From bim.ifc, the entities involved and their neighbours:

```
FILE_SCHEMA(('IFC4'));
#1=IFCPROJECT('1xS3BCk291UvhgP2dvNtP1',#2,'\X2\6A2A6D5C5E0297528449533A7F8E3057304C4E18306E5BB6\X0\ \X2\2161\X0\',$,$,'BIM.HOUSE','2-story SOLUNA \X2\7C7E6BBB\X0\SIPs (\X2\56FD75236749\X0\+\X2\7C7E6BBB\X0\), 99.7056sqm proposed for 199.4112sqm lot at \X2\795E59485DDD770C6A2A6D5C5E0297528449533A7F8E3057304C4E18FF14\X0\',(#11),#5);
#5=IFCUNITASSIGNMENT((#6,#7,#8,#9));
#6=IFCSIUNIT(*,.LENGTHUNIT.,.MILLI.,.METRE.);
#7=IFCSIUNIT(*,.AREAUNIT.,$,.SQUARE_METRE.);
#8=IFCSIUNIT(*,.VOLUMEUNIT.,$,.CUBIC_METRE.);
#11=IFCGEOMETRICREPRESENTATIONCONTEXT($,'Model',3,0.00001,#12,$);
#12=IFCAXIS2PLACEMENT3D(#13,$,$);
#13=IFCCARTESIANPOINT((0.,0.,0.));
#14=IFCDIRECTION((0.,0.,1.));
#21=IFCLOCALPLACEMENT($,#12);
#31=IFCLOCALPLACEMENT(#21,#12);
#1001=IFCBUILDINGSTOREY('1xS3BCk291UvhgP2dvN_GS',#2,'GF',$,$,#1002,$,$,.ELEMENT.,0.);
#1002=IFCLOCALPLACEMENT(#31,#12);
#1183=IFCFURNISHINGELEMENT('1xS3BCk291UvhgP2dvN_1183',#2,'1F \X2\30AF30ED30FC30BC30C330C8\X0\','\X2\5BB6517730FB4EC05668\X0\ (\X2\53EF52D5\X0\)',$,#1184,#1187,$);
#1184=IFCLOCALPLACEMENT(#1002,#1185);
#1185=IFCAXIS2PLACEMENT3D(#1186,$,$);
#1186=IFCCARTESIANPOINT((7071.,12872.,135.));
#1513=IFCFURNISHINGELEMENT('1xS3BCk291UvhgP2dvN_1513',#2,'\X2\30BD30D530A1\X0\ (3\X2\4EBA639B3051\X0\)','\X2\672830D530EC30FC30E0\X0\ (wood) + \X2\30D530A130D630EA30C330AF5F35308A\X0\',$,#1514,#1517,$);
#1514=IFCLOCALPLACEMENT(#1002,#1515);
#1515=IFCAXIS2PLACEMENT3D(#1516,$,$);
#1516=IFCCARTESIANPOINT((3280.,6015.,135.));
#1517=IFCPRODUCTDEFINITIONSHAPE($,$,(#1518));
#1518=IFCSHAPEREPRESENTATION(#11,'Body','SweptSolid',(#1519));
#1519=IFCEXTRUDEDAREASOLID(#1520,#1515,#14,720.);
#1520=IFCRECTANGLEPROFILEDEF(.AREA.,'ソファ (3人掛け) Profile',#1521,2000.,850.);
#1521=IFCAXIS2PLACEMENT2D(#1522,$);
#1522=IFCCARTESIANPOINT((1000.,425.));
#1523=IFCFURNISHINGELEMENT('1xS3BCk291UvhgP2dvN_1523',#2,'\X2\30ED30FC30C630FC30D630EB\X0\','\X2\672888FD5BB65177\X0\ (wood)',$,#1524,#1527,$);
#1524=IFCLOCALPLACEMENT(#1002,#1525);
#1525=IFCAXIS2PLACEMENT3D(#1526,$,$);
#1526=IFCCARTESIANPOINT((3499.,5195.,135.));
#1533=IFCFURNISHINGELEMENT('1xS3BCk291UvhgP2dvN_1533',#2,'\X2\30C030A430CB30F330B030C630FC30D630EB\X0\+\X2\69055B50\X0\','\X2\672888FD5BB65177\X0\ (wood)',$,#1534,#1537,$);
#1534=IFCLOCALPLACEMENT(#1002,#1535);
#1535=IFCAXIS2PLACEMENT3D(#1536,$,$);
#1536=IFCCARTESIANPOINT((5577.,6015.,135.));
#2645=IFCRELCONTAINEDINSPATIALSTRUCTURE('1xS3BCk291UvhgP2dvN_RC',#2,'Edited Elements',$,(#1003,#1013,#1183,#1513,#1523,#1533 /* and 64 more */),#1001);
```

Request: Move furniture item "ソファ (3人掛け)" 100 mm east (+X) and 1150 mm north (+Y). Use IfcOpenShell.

```python
import ifcopenshell
import ifcopenshell.api.geometry
import ifcopenshell.util.placement
import ifcopenshell.util.unit

model = ifcopenshell.open("bim.ifc")
unit_scale = ifcopenshell.util.unit.calculate_unit_scale(model)

item = model.by_guid("1xS3BCk291UvhgP2dvN_1513")
matrix = ifcopenshell.util.placement.get_local_placement(item.ObjectPlacement)
matrix[0, 3] += 0.1 / unit_scale
matrix[1, 3] += 1.15 / unit_scale
ifcopenshell.api.geometry.edit_object_placement(model, product=item, matrix=matrix, is_si=False)

print(ifcopenshell.util.placement.get_local_placement(item.ObjectPlacement).round(3) + 0.0)

model.write("bim_updated.ifc")
```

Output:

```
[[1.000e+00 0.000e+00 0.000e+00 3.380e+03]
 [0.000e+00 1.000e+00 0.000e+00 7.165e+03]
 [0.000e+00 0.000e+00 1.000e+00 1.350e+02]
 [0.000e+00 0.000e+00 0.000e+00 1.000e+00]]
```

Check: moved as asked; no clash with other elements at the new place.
